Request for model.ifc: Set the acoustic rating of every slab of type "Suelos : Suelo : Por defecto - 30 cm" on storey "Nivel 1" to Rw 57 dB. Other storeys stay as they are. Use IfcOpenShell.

First a look at what the model holds.

```python
import ifcopenshell
import ifcopenshell.util.element

model = ifcopenshell.open("model.ifc")
print(model.schema)
storey = next(s for s in model.by_type("IfcBuildingStorey") if s.Name == "Nivel 1")
slabs = [e for e in ifcopenshell.util.element.get_decomposition(storey) if e.is_a("IfcSlab")]
seen = {}
for e in slabs:
    element_type = ifcopenshell.util.element.get_type(e)
    key = (element_type.Name if element_type != e and element_type else None, ifcopenshell.util.element.get_pset(e, "Pset_SlabCommon", "AcousticRating"))
    seen[key] = seen.get(key, 0) + 1
for (name, value), count in sorted(seen.items(), key=str):
    print(count, "x", name, "|", value)
```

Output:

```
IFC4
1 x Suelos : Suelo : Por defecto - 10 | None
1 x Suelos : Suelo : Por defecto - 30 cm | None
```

```python
import ifcopenshell
import ifcopenshell.api.pset
import ifcopenshell.util.element

model = ifcopenshell.open("model.ifc")

storey = next(s for s in model.by_type("IfcBuildingStorey") if s.Name == "Nivel 1")
slabs = [e for e in ifcopenshell.util.element.get_decomposition(storey) if e.is_a("IfcSlab")]

count = 0
for e in slabs:
    element_type = ifcopenshell.util.element.get_type(e)
    if element_type in (None, e) or element_type.Name != "Suelos : Suelo : Por defecto - 30 cm":
        continue
    # add_pset returns the element's existing set when there is one.
    pset = ifcopenshell.api.pset.add_pset(model, product=e, name="Pset_SlabCommon")
    ifcopenshell.api.pset.edit_pset(model, pset=pset, properties={"AcousticRating": "Rw 57 dB"})
    count += 1

print(count, "slabs updated")

model.write("model_edited.ifc")
```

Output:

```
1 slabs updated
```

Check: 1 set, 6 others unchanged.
